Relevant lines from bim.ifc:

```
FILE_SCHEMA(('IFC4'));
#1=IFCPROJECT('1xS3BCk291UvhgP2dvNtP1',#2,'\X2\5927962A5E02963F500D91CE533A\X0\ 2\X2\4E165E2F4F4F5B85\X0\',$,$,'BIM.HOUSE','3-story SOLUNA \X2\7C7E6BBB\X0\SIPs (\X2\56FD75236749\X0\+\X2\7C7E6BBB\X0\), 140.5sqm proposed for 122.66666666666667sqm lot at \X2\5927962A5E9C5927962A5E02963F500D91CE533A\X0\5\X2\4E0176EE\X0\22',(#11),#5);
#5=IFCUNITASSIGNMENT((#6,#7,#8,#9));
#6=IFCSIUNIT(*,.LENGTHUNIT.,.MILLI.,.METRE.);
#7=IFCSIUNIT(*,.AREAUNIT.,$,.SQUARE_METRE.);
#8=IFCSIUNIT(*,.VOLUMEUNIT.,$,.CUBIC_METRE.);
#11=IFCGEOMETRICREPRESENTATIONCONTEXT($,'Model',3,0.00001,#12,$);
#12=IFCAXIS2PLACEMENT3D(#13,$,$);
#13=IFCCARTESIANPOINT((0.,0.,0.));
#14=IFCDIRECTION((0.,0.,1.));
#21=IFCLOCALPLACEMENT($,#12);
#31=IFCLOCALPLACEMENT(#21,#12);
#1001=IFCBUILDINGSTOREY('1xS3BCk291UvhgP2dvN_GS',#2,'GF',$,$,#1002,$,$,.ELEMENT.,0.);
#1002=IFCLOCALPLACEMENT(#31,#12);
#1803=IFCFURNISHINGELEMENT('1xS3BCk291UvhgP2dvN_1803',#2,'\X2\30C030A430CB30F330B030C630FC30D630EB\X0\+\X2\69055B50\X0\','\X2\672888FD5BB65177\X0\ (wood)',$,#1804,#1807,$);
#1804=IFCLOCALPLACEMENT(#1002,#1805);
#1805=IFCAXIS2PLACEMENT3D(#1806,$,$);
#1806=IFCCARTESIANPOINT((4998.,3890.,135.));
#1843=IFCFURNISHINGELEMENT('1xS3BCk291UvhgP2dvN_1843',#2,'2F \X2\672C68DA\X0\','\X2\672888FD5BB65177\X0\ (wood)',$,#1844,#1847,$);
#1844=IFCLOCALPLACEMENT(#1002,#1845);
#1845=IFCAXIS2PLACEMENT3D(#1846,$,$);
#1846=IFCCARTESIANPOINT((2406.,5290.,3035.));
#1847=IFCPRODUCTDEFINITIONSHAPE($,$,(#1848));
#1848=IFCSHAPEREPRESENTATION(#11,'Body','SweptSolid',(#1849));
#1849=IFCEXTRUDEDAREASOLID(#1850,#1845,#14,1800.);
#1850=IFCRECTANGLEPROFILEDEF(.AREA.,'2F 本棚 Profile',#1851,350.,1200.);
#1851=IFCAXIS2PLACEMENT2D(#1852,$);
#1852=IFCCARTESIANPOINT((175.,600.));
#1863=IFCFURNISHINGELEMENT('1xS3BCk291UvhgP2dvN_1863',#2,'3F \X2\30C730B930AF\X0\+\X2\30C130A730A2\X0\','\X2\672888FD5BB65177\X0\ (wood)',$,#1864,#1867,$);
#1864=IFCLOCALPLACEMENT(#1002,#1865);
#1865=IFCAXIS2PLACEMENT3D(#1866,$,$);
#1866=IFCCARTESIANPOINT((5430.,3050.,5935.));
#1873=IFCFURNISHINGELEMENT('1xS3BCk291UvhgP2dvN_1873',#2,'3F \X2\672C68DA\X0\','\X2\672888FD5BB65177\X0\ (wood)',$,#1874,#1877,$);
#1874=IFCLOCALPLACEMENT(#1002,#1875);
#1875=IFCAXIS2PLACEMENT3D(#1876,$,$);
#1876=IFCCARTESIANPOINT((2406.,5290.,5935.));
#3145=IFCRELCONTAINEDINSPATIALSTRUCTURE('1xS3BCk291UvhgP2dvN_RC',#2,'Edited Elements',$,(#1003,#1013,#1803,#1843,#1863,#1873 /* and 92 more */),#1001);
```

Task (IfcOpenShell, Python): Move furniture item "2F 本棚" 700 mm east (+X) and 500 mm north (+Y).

```python
import ifcopenshell
import ifcopenshell.api.geometry
import ifcopenshell.util.placement
import ifcopenshell.util.unit

model = ifcopenshell.open("bim.ifc")
unit_scale = ifcopenshell.util.unit.calculate_unit_scale(model)

item = model.by_guid("1xS3BCk291UvhgP2dvN_1843")
matrix = ifcopenshell.util.placement.get_local_placement(item.ObjectPlacement)
matrix[0, 3] += 0.7 / unit_scale
matrix[1, 3] += 0.5 / unit_scale
ifcopenshell.api.geometry.edit_object_placement(model, product=item, matrix=matrix, is_si=False)

print(ifcopenshell.util.placement.get_local_placement(item.ObjectPlacement).round(3) + 0.0)

model.write("bim-out.ifc")
```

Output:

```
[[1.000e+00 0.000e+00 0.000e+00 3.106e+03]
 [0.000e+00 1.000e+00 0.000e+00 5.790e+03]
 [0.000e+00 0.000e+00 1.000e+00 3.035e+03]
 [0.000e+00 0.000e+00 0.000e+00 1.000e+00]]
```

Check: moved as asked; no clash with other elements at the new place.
